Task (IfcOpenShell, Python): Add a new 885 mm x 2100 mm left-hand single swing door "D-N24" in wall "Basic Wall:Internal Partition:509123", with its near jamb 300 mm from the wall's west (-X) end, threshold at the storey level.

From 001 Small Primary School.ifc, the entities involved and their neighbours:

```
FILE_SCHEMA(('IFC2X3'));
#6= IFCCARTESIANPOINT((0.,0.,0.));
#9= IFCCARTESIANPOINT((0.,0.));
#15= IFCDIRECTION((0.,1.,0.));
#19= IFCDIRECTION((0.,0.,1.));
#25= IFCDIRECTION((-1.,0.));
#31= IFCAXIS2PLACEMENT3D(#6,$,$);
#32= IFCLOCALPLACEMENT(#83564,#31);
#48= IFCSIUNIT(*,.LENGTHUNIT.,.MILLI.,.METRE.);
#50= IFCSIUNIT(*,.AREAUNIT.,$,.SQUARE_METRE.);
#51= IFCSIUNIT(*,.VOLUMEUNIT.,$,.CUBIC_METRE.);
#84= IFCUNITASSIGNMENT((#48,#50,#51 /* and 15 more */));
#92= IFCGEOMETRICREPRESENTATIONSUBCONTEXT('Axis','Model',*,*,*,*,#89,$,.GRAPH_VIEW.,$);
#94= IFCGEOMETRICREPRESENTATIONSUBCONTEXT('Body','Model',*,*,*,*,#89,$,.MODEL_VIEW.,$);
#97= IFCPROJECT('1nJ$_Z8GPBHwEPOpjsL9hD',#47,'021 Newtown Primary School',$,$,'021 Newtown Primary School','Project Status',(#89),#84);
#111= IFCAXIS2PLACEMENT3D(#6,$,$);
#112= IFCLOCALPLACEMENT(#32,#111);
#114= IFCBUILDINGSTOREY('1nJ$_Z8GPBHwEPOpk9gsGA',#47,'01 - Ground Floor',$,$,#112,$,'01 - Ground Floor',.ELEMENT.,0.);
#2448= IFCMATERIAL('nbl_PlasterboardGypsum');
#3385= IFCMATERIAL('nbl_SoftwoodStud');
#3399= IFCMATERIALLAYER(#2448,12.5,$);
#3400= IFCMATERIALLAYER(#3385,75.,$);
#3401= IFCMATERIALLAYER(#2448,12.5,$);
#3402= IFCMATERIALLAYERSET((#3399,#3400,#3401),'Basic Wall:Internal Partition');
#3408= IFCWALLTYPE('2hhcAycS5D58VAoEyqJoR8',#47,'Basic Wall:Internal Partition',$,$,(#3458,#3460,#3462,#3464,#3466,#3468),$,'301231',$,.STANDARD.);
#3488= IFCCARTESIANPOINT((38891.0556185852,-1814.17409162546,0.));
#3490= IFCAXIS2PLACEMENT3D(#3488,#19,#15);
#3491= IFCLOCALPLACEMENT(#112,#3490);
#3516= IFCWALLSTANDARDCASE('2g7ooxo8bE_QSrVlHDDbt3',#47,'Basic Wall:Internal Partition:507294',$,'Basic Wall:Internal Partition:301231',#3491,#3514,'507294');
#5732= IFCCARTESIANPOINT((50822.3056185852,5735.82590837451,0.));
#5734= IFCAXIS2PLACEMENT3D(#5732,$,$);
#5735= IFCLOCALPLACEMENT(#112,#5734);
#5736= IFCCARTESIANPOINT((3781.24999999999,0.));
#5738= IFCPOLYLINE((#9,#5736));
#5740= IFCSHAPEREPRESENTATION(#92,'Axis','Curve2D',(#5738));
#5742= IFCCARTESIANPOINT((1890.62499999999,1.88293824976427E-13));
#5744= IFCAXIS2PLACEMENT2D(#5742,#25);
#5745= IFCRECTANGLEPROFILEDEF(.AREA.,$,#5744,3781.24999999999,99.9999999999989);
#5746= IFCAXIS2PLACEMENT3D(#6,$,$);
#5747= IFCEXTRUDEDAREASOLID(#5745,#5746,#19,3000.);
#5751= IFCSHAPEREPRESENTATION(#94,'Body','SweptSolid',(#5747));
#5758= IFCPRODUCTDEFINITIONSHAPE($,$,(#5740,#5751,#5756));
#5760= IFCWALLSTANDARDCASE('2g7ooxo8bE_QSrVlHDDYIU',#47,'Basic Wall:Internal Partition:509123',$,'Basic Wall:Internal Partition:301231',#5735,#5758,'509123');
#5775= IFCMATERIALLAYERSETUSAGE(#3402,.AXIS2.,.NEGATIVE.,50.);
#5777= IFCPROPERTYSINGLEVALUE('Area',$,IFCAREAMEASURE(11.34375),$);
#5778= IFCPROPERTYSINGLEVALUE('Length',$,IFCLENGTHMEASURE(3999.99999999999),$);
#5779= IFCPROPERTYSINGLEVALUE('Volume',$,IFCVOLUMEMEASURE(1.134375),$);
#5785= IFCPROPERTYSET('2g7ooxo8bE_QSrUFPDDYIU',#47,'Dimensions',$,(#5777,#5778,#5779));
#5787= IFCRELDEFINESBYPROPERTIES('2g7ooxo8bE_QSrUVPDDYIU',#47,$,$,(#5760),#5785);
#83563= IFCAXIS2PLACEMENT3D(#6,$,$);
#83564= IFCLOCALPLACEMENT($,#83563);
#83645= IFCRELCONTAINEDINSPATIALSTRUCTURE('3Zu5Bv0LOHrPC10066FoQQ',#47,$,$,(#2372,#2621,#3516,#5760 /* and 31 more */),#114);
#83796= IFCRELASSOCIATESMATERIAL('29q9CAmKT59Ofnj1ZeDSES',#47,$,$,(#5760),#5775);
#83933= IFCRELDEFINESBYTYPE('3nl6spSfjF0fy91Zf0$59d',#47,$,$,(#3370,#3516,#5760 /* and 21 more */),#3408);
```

```python
import numpy as np
import ifcopenshell
import ifcopenshell.api.feature
import ifcopenshell.api.geometry
import ifcopenshell.api.pset
import ifcopenshell.api.root
import ifcopenshell.api.spatial
import ifcopenshell.api.type
import ifcopenshell.geom
import ifcopenshell.util.element
import ifcopenshell.util.placement
import ifcopenshell.util.representation
import ifcopenshell.util.shape
import ifcopenshell.util.unit

model = ifcopenshell.open("001 Small Primary School.ifc")
unit_scale = ifcopenshell.util.unit.calculate_unit_scale(model)
area_scale = ifcopenshell.util.unit.calculate_unit_scale(model, "AREAUNIT")
volume_scale = ifcopenshell.util.unit.calculate_unit_scale(model, "VOLUMEUNIT")
settings = ifcopenshell.geom.settings()


def volume(element):
    """Net volume in cubic metres, openings subtracted."""
    shape = ifcopenshell.geom.create_shape(settings, element)
    return ifcopenshell.util.shape.get_volume(shape.geometry)


wall = model.by_guid("2g7ooxo8bE_QSrVlHDDYIU")
storey = ifcopenshell.util.element.get_container(wall, ifc_class="IfcBuildingStorey")
context = ifcopenshell.util.representation.get_context(model, "Model", "Body", "MODEL_VIEW")
before = volume(wall)

width, height, from_end, sill = 0.885, 2.1, 0.3, 0.0  # metres

# The wall runs along its own X axis, and the end named is its -X end.
wall_shape = ifcopenshell.geom.create_shape(settings, wall)
x, y, z = ifcopenshell.util.shape.get_vertices(wall_shape.geometry).T
start = x.min() + from_end
face, thickness = float(y.min()), float(y.max() - y.min())
wall_matrix = ifcopenshell.util.placement.get_local_placement(wall.ObjectPlacement)
level = ifcopenshell.util.placement.get_local_placement(storey.ObjectPlacement)[2, 3]


def in_wall(x, y):
    """Placement at x, y metres in the wall's axes, at sill height."""
    matrix = wall_matrix.copy()
    matrix[:, 3] = wall_matrix @ np.array([x / unit_scale, y / unit_scale, 0.0, 1.0])
    matrix[2, 3] = level + sill / unit_scale
    return matrix


# Opening: a box that overshoots both wall faces by 50 mm.
opening = ifcopenshell.api.root.create_entity(model, ifc_class="IfcOpeningElement")
box = ifcopenshell.api.geometry.add_wall_representation(
    model, context=context, length=width, height=height, thickness=thickness + 0.1
)
ifcopenshell.api.geometry.assign_representation(model, product=opening, representation=box)
ifcopenshell.api.geometry.edit_object_placement(model, product=opening, matrix=in_wall(start, face - 0.05), is_si=False)
ifcopenshell.api.feature.add_feature(model, feature=opening, element=wall)

door = ifcopenshell.api.root.create_entity(model, ifc_class="IfcDoor", name="D-N24")
door.OverallWidth, door.OverallHeight = width / unit_scale, height / unit_scale
body = ifcopenshell.api.geometry.add_door_representation(
    model,
    context=context,
    overall_width=door.OverallWidth,
    overall_height=door.OverallHeight,
    operation_type="SINGLE_SWING_LEFT",
    lining_properties={"LiningDepth": thickness / unit_scale, "ThresholdDepth": thickness / unit_scale},
)
ifcopenshell.api.geometry.assign_representation(model, product=door, representation=body)
ifcopenshell.api.spatial.assign_container(model, products=[door], relating_structure=storey)
fills = ifcopenshell.api.feature.add_filling(model, opening=opening, element=door)
fills.OwnerHistory = door.OwnerHistory  # required in IFC2X3

# IFC2X3 keeps the operation on the door style.
style = ifcopenshell.api.root.create_entity(model, ifc_class="IfcDoorStyle", name="D-N24")
style.OperationType, style.ConstructionType = "SINGLE_SWING_LEFT", "NOTDEFINED"
style.ParameterTakesPrecedence = style.Sizeable = False
ifcopenshell.api.type.assign_type(model, related_objects=[door], relating_type=style)

# The lining spans the wall, so the door starts at the wall face.
ifcopenshell.api.geometry.edit_object_placement(model, product=door, matrix=in_wall(start, face), is_si=False)

after = volume(wall)

# Update the wall's stored quantities.
pset = model.by_id(ifcopenshell.util.element.get_pset(wall, "Dimensions", should_inherit=False)["id"])
ifcopenshell.api.pset.edit_pset(model, pset=pset, properties={
    "Area": model.create_entity("IfcAreaMeasure", after / thickness / area_scale),
    "Volume": model.create_entity("IfcVolumeMeasure", after / volume_scale),
})

print(f"wall volume {before:.3f} -> {after:.3f} m3")

model.write("001 Small Primary School_v2.ifc")
```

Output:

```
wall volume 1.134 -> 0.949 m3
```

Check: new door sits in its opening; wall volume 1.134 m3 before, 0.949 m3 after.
